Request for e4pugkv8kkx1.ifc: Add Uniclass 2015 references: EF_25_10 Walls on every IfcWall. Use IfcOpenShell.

First a look at what the model holds.

```python
import ifcopenshell

model = ifcopenshell.open("e4pugkv8kkx1.ifc")
print(model.schema)
print("classifications:", [c.Name for c in model.by_type("IfcClassification")])
for ifc_class in ("IfcDoor", "IfcRoof", "IfcStair", "IfcWall", "IfcWindow"):
    print(ifc_class, len(model.by_type(ifc_class)))
```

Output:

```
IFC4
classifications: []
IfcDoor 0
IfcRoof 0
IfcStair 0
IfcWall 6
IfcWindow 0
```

```python
import ifcopenshell
import ifcopenshell.api.classification

model = ifcopenshell.open("e4pugkv8kkx1.ifc")

system = ifcopenshell.api.classification.add_classification(model, classification="Uniclass 2015")

codes = {
    "IfcWall": ("EF_25_10", "Walls"),
}
for ifc_class, (code, name) in codes.items():
    products = model.by_type(ifc_class)
    ifcopenshell.api.classification.add_reference(
        model, products=products, classification=system, identification=code, name=name
    )
    print(code, len(products))

model.write("e4pugkv8kkx1-out.ifc")
```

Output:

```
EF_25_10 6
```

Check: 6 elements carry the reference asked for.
